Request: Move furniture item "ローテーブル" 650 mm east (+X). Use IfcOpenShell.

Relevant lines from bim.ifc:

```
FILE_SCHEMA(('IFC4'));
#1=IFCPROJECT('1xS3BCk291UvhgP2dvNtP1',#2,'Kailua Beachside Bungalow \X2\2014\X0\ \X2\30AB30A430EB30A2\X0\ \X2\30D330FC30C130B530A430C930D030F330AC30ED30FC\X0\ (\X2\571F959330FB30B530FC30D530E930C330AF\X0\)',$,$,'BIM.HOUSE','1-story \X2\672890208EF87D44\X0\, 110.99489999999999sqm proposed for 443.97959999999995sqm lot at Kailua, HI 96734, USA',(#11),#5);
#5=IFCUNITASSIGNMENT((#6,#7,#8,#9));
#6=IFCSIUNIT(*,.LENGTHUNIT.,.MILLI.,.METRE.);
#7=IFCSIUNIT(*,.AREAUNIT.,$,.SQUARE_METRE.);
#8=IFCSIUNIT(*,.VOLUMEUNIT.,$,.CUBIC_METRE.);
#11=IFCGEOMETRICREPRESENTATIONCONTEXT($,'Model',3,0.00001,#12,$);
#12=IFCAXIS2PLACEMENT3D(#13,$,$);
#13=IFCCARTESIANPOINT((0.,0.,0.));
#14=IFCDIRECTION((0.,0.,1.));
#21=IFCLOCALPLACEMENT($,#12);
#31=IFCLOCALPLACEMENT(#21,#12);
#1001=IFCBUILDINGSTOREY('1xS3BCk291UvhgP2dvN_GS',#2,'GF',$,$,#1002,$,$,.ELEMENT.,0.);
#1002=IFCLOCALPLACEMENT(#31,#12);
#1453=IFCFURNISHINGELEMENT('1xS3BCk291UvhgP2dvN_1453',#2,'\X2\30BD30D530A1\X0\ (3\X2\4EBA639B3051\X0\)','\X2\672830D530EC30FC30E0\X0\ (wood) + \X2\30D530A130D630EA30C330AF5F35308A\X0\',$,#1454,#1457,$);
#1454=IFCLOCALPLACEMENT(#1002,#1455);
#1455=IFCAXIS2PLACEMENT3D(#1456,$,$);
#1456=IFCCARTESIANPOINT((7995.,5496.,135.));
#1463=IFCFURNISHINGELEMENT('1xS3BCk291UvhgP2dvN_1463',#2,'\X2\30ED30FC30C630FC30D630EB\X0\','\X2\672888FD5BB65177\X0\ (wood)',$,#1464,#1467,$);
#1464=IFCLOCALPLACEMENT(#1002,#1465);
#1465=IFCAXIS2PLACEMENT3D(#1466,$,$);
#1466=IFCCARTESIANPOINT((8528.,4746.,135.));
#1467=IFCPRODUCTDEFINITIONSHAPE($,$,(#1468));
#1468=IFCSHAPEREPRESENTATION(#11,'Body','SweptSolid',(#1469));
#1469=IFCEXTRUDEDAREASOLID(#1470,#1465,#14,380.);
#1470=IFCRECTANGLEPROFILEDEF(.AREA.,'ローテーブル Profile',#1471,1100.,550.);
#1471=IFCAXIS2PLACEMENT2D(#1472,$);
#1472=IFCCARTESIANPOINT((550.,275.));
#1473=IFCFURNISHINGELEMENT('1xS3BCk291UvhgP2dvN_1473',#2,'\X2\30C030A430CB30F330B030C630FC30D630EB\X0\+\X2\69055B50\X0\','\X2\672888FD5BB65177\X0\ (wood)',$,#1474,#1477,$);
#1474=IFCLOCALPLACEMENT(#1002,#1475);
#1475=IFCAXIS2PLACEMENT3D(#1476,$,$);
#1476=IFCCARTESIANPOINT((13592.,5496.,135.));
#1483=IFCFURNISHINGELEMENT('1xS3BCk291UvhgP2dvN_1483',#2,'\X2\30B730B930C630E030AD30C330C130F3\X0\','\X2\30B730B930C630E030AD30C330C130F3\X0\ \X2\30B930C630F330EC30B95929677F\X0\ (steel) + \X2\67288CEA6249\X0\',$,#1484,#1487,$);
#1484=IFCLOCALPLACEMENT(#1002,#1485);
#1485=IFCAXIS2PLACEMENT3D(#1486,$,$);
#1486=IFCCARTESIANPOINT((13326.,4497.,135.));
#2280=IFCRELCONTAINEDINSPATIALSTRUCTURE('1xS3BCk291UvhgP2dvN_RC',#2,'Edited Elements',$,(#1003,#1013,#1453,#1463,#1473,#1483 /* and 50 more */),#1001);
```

```python
import ifcopenshell
import ifcopenshell.api.geometry
import ifcopenshell.util.placement
import ifcopenshell.util.unit

model = ifcopenshell.open("bim.ifc")
unit_scale = ifcopenshell.util.unit.calculate_unit_scale(model)

item = model.by_id(1463)
matrix = ifcopenshell.util.placement.get_local_placement(item.ObjectPlacement)
matrix[0, 3] += 0.65 / unit_scale
ifcopenshell.api.geometry.edit_object_placement(model, product=item, matrix=matrix, is_si=False)

print(ifcopenshell.util.placement.get_local_placement(item.ObjectPlacement).round(3) + 0.0)

model.write("bim_updated.ifc")
```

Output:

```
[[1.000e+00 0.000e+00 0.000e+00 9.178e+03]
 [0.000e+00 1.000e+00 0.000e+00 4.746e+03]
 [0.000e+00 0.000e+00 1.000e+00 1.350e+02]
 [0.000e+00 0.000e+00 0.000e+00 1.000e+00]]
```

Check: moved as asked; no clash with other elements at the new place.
